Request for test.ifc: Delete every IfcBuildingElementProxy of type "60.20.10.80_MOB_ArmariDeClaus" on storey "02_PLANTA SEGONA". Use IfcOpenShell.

First a look at what the model holds.

```python
import ifcopenshell
import ifcopenshell.util.element

model = ifcopenshell.open("test.ifc")
print(model.schema)
storey = next(s for s in model.by_type("IfcBuildingStorey") if s.Name == "02_PLANTA SEGONA")
proxies = [e for e in ifcopenshell.util.element.get_decomposition(storey) if e.is_a("IfcBuildingElementProxy")]
seen = {}
for e in proxies:
    element_type = ifcopenshell.util.element.get_type(e)
    name = element_type.Name if element_type not in (None, e) else None
    seen[name] = seen.get(name, 0) + 1
for name, count in sorted(seen.items(), key=str):
    print(count, "x", name)
```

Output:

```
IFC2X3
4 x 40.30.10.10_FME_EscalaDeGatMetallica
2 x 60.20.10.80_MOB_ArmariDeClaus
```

```python
import ifcopenshell
import ifcopenshell.api.root
import ifcopenshell.util.element

model = ifcopenshell.open("test.ifc")

storey = next(s for s in model.by_type("IfcBuildingStorey") if s.Name == "02_PLANTA SEGONA")
proxies = [e for e in ifcopenshell.util.element.get_decomposition(storey) if e.is_a("IfcBuildingElementProxy")]
targets = [e for e in proxies if (t := ifcopenshell.util.element.get_type(e)) not in (None, e) and t.Name == "60.20.10.80_MOB_ArmariDeClaus"]

for e in targets:
    ifcopenshell.api.root.remove_product(model, product=e)
print(len(targets), "removed")

model.write("test-out.ifc")
```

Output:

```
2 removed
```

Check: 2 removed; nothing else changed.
